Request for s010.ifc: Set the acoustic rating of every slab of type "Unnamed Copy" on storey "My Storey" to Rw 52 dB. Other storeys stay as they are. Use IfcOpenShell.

First a look at what the model holds.

```python
import ifcopenshell
import ifcopenshell.util.element

model = ifcopenshell.open("s010.ifc")
print(model.schema)
storey = next(s for s in model.by_type("IfcBuildingStorey") if s.Name == "My Storey")
slabs = [e for e in ifcopenshell.util.element.get_decomposition(storey) if e.is_a("IfcSlab")]
seen = {}
for e in slabs:
    element_type = ifcopenshell.util.element.get_type(e)
    key = (element_type.Name if element_type != e and element_type else None, ifcopenshell.util.element.get_pset(e, "Pset_SlabCommon", "AcousticRating"))
    seen[key] = seen.get(key, 0) + 1
for (name, value), count in sorted(seen.items(), key=str):
    print(count, "x", name, "|", value)
```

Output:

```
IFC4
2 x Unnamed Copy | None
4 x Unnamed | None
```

```python
import ifcopenshell
import ifcopenshell.api.pset
import ifcopenshell.util.element

model = ifcopenshell.open("s010.ifc")

storey = next(s for s in model.by_type("IfcBuildingStorey") if s.Name == "My Storey")
slabs = [e for e in ifcopenshell.util.element.get_decomposition(storey) if e.is_a("IfcSlab")]

count = 0
for e in slabs:
    element_type = ifcopenshell.util.element.get_type(e)
    if element_type in (None, e) or element_type.Name != "Unnamed Copy":
        continue
    # add_pset returns the element's existing set when there is one.
    pset = ifcopenshell.api.pset.add_pset(model, product=e, name="Pset_SlabCommon")
    ifcopenshell.api.pset.edit_pset(model, pset=pset, properties={"AcousticRating": "Rw 52 dB"})
    count += 1

print(count, "slabs updated")

model.write("s010-out.ifc")
```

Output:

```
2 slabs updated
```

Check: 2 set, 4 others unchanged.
